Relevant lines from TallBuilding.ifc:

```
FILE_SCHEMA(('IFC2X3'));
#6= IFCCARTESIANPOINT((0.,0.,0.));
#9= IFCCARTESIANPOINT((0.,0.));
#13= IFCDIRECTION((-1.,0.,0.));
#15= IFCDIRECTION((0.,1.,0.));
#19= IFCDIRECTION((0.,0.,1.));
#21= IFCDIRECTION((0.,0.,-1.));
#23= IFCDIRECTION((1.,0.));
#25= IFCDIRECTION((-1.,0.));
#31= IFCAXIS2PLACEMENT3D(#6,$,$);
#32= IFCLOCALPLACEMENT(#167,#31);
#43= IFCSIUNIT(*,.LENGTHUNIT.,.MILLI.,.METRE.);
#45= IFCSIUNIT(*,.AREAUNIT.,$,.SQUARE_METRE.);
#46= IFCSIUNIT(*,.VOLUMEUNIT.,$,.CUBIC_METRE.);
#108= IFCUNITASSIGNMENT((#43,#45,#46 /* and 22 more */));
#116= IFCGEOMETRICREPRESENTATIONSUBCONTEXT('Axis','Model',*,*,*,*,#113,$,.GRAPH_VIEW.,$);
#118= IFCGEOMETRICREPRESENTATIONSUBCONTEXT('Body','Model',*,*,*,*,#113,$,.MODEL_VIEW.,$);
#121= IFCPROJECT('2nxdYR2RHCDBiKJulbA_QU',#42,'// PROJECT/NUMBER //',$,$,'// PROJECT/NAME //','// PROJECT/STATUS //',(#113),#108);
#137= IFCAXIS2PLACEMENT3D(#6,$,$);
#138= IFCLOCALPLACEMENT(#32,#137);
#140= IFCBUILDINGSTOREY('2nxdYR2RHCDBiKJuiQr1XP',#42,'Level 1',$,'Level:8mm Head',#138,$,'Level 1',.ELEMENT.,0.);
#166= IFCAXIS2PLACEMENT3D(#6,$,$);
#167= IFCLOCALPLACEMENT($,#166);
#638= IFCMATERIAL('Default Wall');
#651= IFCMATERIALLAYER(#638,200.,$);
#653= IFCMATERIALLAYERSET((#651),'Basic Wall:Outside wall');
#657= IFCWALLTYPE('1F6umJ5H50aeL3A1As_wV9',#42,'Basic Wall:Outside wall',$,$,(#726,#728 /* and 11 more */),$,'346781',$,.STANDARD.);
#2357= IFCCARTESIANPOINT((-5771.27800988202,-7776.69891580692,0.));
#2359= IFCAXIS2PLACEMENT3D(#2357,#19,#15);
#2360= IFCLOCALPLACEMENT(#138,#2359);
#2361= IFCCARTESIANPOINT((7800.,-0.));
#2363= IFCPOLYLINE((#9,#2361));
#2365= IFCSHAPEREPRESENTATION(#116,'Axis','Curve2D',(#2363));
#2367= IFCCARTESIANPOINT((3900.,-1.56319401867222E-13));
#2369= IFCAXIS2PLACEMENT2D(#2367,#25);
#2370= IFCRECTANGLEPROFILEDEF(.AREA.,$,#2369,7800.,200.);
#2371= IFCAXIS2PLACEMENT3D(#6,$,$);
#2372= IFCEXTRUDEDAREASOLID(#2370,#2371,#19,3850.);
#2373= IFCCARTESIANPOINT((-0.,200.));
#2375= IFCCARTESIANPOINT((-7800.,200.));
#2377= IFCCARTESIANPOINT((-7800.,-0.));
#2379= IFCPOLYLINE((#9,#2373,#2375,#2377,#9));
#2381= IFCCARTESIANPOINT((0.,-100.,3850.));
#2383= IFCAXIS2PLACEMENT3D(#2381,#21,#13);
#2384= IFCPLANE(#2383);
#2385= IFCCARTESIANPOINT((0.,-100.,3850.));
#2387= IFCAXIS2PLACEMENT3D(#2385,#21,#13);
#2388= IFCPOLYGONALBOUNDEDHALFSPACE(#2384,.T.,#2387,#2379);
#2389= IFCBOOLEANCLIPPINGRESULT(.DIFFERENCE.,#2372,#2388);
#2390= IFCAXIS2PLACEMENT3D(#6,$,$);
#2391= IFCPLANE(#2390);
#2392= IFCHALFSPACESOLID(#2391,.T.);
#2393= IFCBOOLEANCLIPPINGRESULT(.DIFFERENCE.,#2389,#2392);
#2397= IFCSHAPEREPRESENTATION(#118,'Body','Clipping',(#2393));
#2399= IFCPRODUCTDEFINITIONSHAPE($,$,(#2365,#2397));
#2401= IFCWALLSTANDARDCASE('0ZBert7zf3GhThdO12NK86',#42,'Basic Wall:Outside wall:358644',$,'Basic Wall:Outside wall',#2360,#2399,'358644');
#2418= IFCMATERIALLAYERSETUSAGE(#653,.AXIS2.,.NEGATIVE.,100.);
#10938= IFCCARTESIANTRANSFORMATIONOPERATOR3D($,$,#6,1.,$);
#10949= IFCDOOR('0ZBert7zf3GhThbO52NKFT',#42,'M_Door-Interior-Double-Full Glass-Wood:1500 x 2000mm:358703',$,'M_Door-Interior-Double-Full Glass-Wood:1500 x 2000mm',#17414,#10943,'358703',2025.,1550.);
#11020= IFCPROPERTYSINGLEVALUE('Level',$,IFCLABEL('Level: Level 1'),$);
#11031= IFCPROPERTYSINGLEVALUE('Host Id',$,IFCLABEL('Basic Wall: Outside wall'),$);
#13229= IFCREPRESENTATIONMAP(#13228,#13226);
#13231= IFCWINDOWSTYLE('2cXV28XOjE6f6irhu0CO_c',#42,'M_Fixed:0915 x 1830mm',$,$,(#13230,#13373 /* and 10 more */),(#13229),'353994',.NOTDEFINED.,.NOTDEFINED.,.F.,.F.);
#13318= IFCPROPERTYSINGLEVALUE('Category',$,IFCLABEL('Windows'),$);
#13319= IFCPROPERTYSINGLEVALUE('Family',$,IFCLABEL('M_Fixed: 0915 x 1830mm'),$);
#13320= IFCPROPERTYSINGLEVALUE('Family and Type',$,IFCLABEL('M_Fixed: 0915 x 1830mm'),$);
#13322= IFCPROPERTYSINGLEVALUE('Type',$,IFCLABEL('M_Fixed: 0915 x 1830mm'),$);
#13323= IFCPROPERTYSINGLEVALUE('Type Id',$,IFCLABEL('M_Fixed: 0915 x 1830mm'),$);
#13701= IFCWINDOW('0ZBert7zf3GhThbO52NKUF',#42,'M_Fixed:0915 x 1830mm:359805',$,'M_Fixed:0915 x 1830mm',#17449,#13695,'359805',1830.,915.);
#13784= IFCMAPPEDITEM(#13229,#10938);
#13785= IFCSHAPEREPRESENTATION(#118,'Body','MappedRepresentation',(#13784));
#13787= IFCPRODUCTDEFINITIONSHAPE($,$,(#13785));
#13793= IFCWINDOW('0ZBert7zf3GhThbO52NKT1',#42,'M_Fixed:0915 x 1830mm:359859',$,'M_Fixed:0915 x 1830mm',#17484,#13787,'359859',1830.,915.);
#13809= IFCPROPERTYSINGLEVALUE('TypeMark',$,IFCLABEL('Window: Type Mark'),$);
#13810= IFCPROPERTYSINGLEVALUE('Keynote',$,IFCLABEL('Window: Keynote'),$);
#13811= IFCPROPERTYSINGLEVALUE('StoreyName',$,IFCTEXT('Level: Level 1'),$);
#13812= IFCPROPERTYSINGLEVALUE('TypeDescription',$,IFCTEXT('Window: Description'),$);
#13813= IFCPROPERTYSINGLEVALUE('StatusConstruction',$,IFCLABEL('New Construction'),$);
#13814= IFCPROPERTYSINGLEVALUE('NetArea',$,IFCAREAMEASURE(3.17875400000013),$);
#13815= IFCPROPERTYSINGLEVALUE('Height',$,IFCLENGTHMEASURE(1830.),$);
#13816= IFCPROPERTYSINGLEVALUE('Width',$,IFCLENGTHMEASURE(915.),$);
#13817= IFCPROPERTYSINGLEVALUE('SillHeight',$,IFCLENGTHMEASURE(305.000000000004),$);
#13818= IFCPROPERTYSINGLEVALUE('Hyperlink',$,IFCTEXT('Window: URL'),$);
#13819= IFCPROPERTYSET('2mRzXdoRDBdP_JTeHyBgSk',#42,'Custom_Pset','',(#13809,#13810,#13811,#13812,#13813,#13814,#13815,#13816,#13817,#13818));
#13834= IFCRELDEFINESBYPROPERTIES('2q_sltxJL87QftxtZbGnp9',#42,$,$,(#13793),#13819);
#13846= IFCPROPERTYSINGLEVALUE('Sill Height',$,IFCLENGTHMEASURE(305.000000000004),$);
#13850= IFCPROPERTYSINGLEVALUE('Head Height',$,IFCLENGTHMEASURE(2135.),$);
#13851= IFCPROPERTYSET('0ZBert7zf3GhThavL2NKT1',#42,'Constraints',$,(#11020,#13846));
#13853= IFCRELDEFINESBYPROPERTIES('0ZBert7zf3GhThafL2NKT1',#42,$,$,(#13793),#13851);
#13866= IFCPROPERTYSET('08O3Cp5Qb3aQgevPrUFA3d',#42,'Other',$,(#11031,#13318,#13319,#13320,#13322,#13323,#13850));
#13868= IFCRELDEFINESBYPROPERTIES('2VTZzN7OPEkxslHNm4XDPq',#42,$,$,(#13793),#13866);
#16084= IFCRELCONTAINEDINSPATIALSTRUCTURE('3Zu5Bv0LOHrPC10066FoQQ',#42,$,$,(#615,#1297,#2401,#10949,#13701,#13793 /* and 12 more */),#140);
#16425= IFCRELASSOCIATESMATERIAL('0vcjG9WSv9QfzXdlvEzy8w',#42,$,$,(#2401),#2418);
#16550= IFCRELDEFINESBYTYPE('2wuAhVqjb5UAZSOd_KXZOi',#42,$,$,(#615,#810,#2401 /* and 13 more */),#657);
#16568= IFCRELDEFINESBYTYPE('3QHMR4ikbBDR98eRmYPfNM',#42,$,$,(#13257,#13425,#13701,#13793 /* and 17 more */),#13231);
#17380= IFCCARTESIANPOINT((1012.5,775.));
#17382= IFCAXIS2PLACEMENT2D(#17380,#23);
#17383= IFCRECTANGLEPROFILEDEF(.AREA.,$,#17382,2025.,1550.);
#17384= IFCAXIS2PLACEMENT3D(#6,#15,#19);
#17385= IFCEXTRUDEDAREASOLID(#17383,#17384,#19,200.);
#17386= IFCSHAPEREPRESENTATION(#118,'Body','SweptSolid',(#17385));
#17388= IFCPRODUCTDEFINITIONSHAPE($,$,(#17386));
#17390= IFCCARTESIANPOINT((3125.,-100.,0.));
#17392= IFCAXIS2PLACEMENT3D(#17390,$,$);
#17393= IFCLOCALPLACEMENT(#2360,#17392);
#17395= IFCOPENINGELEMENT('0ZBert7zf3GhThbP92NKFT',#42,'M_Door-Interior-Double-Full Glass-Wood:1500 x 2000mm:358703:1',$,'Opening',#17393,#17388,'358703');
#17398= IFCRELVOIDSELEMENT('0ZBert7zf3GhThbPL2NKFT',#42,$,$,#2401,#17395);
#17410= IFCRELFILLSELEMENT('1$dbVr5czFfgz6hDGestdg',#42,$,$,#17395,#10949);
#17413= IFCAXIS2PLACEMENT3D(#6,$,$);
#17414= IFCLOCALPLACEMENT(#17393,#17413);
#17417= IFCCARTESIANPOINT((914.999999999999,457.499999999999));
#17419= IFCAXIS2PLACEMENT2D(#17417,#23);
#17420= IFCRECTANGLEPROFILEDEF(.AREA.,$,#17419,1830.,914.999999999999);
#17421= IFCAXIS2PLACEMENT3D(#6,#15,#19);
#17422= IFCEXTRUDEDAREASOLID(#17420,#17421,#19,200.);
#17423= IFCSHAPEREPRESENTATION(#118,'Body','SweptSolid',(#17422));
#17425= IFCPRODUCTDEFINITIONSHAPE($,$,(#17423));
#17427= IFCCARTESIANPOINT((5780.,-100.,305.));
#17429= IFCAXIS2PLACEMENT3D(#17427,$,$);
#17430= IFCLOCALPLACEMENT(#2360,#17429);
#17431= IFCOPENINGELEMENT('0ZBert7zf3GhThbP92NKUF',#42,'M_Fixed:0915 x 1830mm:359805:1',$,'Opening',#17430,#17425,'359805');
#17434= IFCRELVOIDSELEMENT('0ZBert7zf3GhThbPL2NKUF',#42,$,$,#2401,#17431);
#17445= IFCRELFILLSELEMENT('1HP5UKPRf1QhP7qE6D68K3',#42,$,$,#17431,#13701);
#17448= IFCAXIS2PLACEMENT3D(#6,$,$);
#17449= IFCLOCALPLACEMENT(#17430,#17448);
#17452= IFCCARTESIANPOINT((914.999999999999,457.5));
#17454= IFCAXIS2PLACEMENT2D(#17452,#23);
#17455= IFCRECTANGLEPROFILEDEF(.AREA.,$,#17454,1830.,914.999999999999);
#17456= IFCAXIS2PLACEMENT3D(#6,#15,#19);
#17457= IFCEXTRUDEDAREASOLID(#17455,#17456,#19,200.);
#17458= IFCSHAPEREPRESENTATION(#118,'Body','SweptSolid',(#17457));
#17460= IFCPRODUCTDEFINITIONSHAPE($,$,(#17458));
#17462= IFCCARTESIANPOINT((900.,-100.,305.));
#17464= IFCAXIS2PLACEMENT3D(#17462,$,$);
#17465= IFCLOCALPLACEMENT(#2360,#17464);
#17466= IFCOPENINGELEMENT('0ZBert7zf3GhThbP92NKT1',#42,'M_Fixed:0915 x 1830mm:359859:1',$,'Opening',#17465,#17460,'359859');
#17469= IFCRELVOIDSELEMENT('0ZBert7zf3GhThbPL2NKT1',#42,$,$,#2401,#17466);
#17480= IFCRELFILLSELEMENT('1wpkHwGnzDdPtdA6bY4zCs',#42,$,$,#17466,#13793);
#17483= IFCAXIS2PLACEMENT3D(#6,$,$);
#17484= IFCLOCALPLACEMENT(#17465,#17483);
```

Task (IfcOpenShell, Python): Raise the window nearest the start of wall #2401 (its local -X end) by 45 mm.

```python
import numpy as np
import ifcopenshell
import ifcopenshell.api.geometry
import ifcopenshell.api.pset
import ifcopenshell.util.element
import ifcopenshell.util.placement
import ifcopenshell.util.unit

model = ifcopenshell.open("TallBuilding.ifc")
unit_scale = ifcopenshell.util.unit.calculate_unit_scale(model)

window = model.by_guid("0ZBert7zf3GhThbO52NKT1")
opening = window.FillsVoids[0].RelatingOpeningElement
dz = 45.0

shift = np.array([0.0, 0.0, dz])
# The window is placed relative to its opening, so it follows when the opening moves.
matrix = ifcopenshell.util.placement.get_local_placement(opening.ObjectPlacement)
matrix[:3, 3] += shift
ifcopenshell.api.geometry.edit_object_placement(
    model, product=opening, matrix=matrix, is_si=False, should_transform_children=True
)

# Keep the stored heights in step.
pset = model.by_id(ifcopenshell.util.element.get_pset(window, "Custom_Pset", should_inherit=False)["id"])
ifcopenshell.api.pset.edit_pset(model, pset=pset, properties={
    "SillHeight": model.create_entity("IfcLengthMeasure", ifcopenshell.util.element.get_pset(window, "Constraints", "Sill Height") + dz),
})
pset = model.by_id(ifcopenshell.util.element.get_pset(window, "Constraints", should_inherit=False)["id"])
ifcopenshell.api.pset.edit_pset(model, pset=pset, properties={
    "Sill Height": model.create_entity("IfcLengthMeasure", ifcopenshell.util.element.get_pset(window, "Constraints", "Sill Height") + dz),
})
pset = model.by_id(ifcopenshell.util.element.get_pset(window, "Other", should_inherit=False)["id"])
ifcopenshell.api.pset.edit_pset(model, pset=pset, properties={
    "Head Height": model.create_entity("IfcLengthMeasure", ifcopenshell.util.element.get_pset(window, "Other", "Head Height") + dz),
})

print(f"moved by {dz * unit_scale:+.3f} m")

model.write("TallBuilding_rev.ifc")
```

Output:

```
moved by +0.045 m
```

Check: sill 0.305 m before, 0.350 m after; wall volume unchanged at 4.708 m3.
